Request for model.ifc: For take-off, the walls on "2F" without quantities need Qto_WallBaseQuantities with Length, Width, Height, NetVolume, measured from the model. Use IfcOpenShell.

First a look at what the model holds.

```python
import ifcopenshell
import ifcopenshell.util.element
import ifcopenshell.util.unit

model = ifcopenshell.open("model.ifc")
print(model.schema)
for unit_type in ("LENGTHUNIT", "AREAUNIT", "VOLUMEUNIT"):
    print(unit_type, ifcopenshell.util.unit.calculate_unit_scale(model, unit_type))
storey = next(s for s in model.by_type("IfcBuildingStorey") if s.Name == "2F")
walls = [e for e in ifcopenshell.util.element.get_decomposition(storey) if e.is_a("IfcWall")]
for e in sorted(walls, key=lambda e: e.id()):
    print(e.id(), e.is_a(), e.Name, list(ifcopenshell.util.element.get_psets(e, qtos_only=True)), sep=" | ")
```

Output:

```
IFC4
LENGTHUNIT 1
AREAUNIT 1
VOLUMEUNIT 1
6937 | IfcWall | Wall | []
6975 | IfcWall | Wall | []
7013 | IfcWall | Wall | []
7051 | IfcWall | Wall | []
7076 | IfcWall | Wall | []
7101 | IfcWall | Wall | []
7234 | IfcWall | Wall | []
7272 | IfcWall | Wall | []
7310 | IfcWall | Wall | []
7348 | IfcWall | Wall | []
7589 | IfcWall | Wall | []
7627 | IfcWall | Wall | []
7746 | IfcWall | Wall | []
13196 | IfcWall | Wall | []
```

```python
import ifcopenshell
import ifcopenshell.api.pset
import ifcopenshell.geom
import ifcopenshell.util.element
import ifcopenshell.util.shape
import ifcopenshell.util.unit

model = ifcopenshell.open("model.ifc")
unit_scale = ifcopenshell.util.unit.calculate_unit_scale(model)
volume_scale = ifcopenshell.util.unit.calculate_unit_scale(model, "VOLUMEUNIT")
settings = ifcopenshell.geom.settings()

storey = next(s for s in model.by_type("IfcBuildingStorey") if s.Name == "2F")
walls = [e for e in ifcopenshell.util.element.get_decomposition(storey) if e.is_a("IfcWall")]

for e in sorted(walls, key=lambda e: e.id()):
    if ifcopenshell.util.element.get_psets(e, qtos_only=True, should_inherit=False):
        continue
    # Geometry comes back in metres, in the element's own axes.
    shape = ifcopenshell.geom.create_shape(settings, e)
    values = {
        "Length": ifcopenshell.util.shape.get_x(shape.geometry) / unit_scale,
        "Width": ifcopenshell.util.shape.get_y(shape.geometry) / unit_scale,
        "Height": ifcopenshell.util.shape.get_z(shape.geometry) / unit_scale,
        "NetVolume": ifcopenshell.util.shape.get_volume(shape.geometry) / volume_scale,
    }
    qto = ifcopenshell.api.pset.add_qto(model, product=e, name="Qto_WallBaseQuantities")
    ifcopenshell.api.pset.edit_qto(model, qto=qto, properties=values)
    print(e.id(), {k: round(v, 3) for k, v in values.items()})

model.write("model_updated.ifc")
```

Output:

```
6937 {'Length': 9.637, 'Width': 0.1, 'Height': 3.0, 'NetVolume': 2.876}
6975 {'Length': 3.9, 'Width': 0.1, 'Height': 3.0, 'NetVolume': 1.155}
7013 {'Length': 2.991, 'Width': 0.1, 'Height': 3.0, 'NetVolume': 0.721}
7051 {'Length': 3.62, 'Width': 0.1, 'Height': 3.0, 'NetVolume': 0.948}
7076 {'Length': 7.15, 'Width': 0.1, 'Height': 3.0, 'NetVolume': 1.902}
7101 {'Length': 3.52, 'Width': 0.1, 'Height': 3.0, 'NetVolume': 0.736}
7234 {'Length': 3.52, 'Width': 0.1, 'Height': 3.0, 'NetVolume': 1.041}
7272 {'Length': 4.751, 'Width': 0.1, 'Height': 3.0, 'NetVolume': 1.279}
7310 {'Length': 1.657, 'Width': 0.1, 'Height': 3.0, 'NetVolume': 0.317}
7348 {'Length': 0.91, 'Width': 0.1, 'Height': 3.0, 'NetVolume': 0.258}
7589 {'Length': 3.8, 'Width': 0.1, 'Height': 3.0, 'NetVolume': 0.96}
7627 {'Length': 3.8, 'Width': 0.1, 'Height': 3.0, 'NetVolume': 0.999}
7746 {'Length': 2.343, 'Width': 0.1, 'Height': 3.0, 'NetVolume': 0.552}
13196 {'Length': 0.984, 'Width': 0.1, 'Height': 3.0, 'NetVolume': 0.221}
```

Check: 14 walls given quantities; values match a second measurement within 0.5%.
